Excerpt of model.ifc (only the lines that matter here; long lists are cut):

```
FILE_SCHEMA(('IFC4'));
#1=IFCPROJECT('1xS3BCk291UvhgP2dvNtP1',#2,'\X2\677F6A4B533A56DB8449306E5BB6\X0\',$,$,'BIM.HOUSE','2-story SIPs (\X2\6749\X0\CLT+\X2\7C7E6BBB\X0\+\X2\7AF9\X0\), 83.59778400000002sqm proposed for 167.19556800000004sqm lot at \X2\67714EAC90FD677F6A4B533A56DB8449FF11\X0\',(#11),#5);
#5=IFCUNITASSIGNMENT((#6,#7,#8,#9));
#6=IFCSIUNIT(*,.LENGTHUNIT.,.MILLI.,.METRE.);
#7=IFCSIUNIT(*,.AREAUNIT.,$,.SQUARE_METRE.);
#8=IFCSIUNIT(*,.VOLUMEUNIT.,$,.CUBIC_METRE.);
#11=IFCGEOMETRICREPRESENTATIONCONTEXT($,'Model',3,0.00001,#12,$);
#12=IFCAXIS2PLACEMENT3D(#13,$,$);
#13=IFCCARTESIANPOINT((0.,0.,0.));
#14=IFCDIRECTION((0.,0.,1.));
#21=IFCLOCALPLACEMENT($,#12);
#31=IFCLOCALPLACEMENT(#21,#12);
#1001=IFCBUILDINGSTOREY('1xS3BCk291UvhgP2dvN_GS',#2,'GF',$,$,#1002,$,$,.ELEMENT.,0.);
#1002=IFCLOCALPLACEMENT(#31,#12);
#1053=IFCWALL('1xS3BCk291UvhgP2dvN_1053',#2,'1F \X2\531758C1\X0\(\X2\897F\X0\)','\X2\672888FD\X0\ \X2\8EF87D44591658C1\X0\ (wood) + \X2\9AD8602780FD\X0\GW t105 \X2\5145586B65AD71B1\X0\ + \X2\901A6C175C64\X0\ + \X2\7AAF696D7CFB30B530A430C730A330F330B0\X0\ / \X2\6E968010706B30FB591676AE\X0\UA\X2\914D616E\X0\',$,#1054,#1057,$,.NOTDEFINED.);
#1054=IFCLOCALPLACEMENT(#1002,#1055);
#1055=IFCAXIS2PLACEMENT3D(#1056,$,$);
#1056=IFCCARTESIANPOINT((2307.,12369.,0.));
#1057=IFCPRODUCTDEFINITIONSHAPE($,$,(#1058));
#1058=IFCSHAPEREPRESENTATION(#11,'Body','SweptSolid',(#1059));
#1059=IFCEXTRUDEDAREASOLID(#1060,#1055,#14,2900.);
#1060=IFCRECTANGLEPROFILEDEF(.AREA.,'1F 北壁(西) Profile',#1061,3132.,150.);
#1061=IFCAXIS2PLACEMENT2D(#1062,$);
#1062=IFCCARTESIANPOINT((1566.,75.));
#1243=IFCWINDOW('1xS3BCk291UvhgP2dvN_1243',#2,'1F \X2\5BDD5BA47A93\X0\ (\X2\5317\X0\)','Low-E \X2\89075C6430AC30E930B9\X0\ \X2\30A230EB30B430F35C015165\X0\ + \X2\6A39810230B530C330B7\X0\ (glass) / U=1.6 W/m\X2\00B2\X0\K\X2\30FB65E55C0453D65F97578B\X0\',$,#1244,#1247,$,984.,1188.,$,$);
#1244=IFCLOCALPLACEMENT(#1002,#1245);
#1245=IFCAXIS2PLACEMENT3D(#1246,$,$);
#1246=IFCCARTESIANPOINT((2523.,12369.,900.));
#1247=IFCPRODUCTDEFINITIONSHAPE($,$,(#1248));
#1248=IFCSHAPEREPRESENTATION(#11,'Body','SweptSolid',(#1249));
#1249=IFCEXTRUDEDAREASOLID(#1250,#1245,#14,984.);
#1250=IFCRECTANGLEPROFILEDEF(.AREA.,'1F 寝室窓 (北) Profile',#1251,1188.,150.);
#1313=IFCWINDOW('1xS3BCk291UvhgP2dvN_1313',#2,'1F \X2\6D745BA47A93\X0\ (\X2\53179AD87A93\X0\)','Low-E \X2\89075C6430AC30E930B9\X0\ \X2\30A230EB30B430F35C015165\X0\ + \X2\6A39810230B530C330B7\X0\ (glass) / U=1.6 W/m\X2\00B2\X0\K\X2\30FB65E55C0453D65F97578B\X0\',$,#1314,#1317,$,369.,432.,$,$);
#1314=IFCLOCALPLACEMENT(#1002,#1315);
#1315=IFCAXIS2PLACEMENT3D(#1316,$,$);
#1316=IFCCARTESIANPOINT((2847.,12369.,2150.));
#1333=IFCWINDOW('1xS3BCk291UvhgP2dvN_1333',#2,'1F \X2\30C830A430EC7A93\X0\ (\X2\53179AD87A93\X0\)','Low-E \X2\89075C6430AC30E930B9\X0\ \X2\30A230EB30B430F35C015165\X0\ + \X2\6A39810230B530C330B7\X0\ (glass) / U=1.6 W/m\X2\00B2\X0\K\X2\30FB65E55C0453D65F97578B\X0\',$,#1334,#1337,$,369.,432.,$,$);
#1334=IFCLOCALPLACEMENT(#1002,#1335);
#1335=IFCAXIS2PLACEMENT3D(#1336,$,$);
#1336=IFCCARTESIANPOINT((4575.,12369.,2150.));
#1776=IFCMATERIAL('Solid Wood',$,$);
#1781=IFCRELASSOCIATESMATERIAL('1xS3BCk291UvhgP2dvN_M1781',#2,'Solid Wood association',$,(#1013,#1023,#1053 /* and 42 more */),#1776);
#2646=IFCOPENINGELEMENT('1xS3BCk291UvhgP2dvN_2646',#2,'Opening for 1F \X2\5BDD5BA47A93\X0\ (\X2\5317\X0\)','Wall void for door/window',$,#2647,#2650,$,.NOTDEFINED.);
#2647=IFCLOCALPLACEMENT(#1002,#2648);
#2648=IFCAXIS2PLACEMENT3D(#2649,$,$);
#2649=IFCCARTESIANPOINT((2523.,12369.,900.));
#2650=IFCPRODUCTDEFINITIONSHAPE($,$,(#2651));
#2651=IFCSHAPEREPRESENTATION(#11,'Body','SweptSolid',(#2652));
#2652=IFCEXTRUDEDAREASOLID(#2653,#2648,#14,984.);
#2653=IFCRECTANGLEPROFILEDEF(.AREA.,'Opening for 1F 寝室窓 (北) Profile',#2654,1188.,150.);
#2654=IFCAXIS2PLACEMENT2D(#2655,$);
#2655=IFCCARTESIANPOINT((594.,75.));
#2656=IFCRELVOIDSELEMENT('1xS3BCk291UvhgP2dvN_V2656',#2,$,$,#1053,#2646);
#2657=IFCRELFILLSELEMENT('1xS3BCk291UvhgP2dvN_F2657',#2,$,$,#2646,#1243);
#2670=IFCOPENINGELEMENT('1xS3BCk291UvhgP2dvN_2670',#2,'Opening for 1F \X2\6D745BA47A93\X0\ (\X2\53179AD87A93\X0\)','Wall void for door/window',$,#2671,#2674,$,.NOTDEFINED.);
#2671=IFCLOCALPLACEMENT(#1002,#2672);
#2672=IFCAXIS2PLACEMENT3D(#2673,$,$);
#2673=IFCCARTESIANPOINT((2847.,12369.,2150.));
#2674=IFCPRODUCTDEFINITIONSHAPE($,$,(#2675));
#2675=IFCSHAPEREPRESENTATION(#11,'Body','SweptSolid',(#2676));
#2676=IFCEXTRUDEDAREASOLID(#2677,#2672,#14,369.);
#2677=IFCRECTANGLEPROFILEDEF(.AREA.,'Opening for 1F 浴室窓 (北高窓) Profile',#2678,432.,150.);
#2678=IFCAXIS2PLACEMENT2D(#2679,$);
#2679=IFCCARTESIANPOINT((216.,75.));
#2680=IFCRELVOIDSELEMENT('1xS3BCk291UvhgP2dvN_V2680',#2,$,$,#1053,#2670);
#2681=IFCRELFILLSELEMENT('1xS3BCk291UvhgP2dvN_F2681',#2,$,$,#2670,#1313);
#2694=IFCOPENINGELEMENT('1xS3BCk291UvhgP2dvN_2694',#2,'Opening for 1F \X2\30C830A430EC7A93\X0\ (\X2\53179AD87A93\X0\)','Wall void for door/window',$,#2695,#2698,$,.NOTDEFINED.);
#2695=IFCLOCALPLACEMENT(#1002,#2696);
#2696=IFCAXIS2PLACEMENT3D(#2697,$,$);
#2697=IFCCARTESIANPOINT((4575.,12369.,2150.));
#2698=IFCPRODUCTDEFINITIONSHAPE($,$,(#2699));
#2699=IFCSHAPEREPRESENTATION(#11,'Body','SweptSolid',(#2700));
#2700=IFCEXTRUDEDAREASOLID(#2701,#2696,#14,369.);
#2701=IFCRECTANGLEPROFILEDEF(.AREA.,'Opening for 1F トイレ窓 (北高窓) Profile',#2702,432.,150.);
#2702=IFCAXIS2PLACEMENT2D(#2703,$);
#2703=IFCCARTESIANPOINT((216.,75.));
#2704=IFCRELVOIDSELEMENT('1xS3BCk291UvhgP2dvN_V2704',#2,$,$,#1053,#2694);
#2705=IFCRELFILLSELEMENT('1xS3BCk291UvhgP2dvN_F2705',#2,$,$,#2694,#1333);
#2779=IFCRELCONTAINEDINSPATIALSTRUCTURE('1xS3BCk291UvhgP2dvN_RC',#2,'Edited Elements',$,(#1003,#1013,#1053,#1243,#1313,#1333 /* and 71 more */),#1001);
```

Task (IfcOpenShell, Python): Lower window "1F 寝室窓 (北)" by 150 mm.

```python
import numpy as np
import ifcopenshell
import ifcopenshell.api.geometry
import ifcopenshell.util.placement
import ifcopenshell.util.unit

model = ifcopenshell.open("model.ifc")
unit_scale = ifcopenshell.util.unit.calculate_unit_scale(model)

window = model.by_id(1243)
opening = window.FillsVoids[0].RelatingOpeningElement
dz = -0.15 / unit_scale

shift = np.array([0.0, 0.0, dz])
# The window is not placed relative to its opening, so move both.
for product in (opening, window):
    matrix = ifcopenshell.util.placement.get_local_placement(product.ObjectPlacement)
    matrix[:3, 3] += shift
    ifcopenshell.api.geometry.edit_object_placement(model, product=product, matrix=matrix, is_si=False)

print(f"moved by {dz * unit_scale:+.3f} m")

model.write("model_edited.ifc")
```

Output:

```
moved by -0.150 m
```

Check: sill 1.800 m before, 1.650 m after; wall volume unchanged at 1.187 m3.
